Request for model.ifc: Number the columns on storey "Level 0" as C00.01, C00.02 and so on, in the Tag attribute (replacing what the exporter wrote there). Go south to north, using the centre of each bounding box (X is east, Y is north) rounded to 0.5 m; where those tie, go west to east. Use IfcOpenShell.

First a look at what the model holds.

```python
import ifcopenshell
import ifcopenshell.util.element
import ifcopenshell.util.placement

model = ifcopenshell.open("model.ifc")
print(model.schema)
storey = next(s for s in model.by_type("IfcBuildingStorey") if s.Name == "Level 0")
columns = [e for e in ifcopenshell.util.element.get_decomposition(storey) if e.is_a("IfcColumn")]
for e in sorted(columns, key=lambda e: e.id()):
    origin = ifcopenshell.util.placement.get_local_placement(e.ObjectPlacement)[:3, 3]
    print(e.id(), e.Tag, e.Name, origin.round(2) + 0.0, sep=" | ")
```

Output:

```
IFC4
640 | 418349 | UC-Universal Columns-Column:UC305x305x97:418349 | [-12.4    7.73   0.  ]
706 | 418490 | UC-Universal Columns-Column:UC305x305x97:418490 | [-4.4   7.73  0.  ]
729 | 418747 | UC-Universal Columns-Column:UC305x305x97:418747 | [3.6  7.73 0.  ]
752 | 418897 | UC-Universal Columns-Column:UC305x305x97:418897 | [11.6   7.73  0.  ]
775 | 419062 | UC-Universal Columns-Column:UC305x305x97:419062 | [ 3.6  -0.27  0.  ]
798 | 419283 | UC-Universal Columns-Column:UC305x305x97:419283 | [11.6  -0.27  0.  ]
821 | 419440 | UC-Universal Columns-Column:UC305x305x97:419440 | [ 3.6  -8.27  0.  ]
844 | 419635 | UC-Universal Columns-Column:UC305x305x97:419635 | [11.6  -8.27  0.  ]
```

```python
import ifcopenshell
import ifcopenshell.geom
import ifcopenshell.util.element
import ifcopenshell.util.shape

model = ifcopenshell.open("model.ifc")
settings = ifcopenshell.geom.settings()
settings.set("use-world-coords", True)


def centre(element):
    shape = ifcopenshell.geom.create_shape(settings, element)
    return ifcopenshell.util.shape.get_bbox_centroid(shape.geometry)


storey = next(s for s in model.by_type("IfcBuildingStorey") if s.Name == "Level 0")
columns = [e for e in ifcopenshell.util.element.get_decomposition(storey) if e.is_a("IfcColumn")]

# Insertion points can sit at a corner or the storey origin, so sort by the geometry (in metres).
centres = {e: centre(e) for e in columns}
columns.sort(key=lambda e: (round(centres[e][1] / 0.5), centres[e][0]))

for i, e in enumerate(columns, start=1):
    number = f"C00.{i:02d}"
    e.Tag = number
    print(e.id(), number)

model.write("model_v2.ifc")
```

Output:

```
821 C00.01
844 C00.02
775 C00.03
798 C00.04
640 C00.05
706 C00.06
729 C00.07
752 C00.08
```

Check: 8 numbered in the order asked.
